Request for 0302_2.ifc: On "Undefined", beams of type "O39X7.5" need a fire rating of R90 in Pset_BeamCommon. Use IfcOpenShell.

First a look at what the model holds.

```python
import ifcopenshell
import ifcopenshell.util.element

model = ifcopenshell.open("0302_2.ifc")
print(model.schema)
storey = next(s for s in model.by_type("IfcBuildingStorey") if s.Name == "Undefined")
beams = [e for e in ifcopenshell.util.element.get_decomposition(storey) if e.is_a("IfcBeam")]
seen = {}
for e in beams:
    element_type = ifcopenshell.util.element.get_type(e)
    key = (element_type.Name if element_type != e and element_type else None, ifcopenshell.util.element.get_pset(e, "Pset_BeamCommon", "FireRating"))
    seen[key] = seen.get(key, 0) + 1
for (name, value), count in sorted(seen.items(), key=str):
    print(count, "x", name, "|", value)
```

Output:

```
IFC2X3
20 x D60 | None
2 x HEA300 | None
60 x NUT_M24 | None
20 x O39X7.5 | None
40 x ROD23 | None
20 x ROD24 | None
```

```python
import ifcopenshell
import ifcopenshell.api.pset
import ifcopenshell.util.element

model = ifcopenshell.open("0302_2.ifc")

storey = next(s for s in model.by_type("IfcBuildingStorey") if s.Name == "Undefined")
beams = [e for e in ifcopenshell.util.element.get_decomposition(storey) if e.is_a("IfcBeam")]

count = 0
for e in beams:
    element_type = ifcopenshell.util.element.get_type(e)
    if element_type in (None, e) or element_type.Name != "O39X7.5":
        continue
    found = ifcopenshell.util.element.get_pset(e, "Pset_BeamCommon", should_inherit=False)
    if found:
        pset = model.by_id(found["id"])
        if len(ifcopenshell.util.element.get_elements_by_pset(pset)) > 1:
            pset = ifcopenshell.api.pset.unshare_pset(model, products=[e], pset=pset)[0]
    else:
        pset = ifcopenshell.api.pset.add_pset(model, product=e, name="Pset_BeamCommon")
    ifcopenshell.api.pset.edit_pset(model, pset=pset, properties={"FireRating": "R90"})
    count += 1

print(count, "beams updated")

model.write("0302_2_edited.ifc")
```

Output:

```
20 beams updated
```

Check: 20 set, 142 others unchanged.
